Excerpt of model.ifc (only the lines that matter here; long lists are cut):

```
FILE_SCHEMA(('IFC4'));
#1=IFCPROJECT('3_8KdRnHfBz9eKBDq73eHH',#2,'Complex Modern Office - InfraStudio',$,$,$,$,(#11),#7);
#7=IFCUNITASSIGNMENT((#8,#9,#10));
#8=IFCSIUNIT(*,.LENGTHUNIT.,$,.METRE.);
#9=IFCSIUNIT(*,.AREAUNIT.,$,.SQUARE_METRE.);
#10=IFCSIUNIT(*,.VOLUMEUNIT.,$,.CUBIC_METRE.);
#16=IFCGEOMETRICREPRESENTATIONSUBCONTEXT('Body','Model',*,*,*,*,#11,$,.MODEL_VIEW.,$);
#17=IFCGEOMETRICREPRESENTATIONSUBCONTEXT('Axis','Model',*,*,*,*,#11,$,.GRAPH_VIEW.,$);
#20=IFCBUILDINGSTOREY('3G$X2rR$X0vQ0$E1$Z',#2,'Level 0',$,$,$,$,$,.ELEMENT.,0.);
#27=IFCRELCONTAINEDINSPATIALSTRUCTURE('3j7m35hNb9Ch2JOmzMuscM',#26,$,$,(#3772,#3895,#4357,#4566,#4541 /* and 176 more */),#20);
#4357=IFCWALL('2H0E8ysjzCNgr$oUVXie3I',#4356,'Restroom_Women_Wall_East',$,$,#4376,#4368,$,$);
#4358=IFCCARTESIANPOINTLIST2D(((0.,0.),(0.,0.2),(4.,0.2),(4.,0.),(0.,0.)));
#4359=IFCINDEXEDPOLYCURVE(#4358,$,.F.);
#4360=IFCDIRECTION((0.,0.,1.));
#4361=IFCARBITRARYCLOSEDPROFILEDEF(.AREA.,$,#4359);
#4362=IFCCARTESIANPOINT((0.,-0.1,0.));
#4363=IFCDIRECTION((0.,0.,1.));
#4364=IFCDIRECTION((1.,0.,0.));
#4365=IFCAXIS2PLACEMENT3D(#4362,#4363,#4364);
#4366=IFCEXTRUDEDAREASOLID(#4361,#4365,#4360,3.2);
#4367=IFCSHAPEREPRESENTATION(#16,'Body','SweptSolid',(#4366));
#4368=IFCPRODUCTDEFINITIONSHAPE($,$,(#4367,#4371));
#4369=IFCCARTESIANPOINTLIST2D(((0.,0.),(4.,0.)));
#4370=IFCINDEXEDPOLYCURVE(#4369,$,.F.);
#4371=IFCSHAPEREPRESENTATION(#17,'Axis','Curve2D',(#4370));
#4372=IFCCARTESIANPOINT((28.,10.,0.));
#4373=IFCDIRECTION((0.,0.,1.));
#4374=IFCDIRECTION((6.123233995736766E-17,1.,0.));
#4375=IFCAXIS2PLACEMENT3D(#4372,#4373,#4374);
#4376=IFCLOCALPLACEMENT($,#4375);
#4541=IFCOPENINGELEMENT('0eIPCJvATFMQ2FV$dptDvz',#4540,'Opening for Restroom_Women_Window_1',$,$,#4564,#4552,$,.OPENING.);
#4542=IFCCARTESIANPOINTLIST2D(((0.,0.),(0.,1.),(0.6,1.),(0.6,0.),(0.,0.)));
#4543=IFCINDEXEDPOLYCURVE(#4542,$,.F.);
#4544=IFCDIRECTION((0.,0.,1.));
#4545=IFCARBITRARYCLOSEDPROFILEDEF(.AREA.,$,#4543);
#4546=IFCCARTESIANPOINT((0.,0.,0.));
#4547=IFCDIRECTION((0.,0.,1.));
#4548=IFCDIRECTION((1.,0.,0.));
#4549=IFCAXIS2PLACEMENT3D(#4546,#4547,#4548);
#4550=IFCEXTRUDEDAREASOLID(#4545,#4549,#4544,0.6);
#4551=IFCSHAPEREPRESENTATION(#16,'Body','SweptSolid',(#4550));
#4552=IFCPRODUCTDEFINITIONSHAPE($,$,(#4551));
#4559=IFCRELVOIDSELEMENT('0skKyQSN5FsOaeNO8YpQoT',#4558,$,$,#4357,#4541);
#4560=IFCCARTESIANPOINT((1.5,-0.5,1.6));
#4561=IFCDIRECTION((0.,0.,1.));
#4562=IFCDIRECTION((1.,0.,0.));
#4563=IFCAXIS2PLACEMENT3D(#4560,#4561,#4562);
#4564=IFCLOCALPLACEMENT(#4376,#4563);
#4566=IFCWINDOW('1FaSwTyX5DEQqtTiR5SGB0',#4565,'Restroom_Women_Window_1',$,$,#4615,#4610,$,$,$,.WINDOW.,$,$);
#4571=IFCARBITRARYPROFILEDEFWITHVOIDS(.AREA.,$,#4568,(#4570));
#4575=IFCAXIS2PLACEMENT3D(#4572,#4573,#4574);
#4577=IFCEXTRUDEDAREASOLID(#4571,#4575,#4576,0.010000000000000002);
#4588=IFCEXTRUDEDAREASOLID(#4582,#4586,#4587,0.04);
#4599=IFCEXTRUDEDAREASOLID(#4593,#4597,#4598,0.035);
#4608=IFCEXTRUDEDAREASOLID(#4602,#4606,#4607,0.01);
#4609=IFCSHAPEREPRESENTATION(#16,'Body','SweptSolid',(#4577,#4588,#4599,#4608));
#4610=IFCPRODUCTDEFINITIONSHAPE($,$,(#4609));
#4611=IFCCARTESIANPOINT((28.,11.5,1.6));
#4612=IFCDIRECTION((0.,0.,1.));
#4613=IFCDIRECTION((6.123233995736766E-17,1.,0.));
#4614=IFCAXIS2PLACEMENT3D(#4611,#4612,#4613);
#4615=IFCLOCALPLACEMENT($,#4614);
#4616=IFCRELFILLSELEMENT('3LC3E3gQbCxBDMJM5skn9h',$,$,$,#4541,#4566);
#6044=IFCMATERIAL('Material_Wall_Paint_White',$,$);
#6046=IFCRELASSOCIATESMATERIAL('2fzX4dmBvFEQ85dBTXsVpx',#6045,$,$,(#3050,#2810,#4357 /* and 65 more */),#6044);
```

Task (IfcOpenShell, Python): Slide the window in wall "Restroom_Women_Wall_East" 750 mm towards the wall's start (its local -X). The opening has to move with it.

```python
import ifcopenshell
import ifcopenshell.api.geometry
import ifcopenshell.util.placement
import ifcopenshell.util.unit

model = ifcopenshell.open("model.ifc")
unit_scale = ifcopenshell.util.unit.calculate_unit_scale(model)

window = model.by_id(4566)
opening = window.FillsVoids[0].RelatingOpeningElement
wall = opening.VoidsElements[0].RelatingBuildingElement

wall_matrix = ifcopenshell.util.placement.get_local_placement(wall.ObjectPlacement)
shift = wall_matrix[:3, 0] * -0.75 / unit_scale
before = ifcopenshell.util.placement.get_local_placement(window.ObjectPlacement)[:3, 3].copy()

# The window is not placed relative to its opening, so move both.
for product in (opening, window):
    matrix = ifcopenshell.util.placement.get_local_placement(product.ObjectPlacement)
    matrix[:3, 3] += shift
    ifcopenshell.api.geometry.edit_object_placement(model, product=product, matrix=matrix, is_si=False)

after = ifcopenshell.util.placement.get_local_placement(window.ObjectPlacement)[:3, 3]
print("window moved by", (after - before).round(3) + 0.0)

model.write("model-out.ifc")
```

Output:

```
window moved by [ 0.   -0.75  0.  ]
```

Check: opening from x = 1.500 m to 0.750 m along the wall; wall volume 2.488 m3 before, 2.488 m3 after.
